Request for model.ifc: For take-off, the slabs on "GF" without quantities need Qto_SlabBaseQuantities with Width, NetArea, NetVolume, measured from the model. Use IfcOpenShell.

First a look at what the model holds.

```python
import ifcopenshell
import ifcopenshell.util.element
import ifcopenshell.util.unit

model = ifcopenshell.open("model.ifc")
print(model.schema)
for unit_type in ("LENGTHUNIT", "AREAUNIT", "VOLUMEUNIT"):
    print(unit_type, ifcopenshell.util.unit.calculate_unit_scale(model, unit_type))
storey = next(s for s in model.by_type("IfcBuildingStorey") if s.Name == "GF")
slabs = [e for e in ifcopenshell.util.element.get_decomposition(storey) if e.is_a("IfcSlab")]
for e in sorted(slabs, key=lambda e: e.id()):
    print(e.id(), e.is_a(), e.Name, list(ifcopenshell.util.element.get_psets(e, qtos_only=True)), sep=" | ")
```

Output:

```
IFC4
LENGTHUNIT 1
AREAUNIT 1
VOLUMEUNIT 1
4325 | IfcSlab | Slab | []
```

```python
import ifcopenshell
import ifcopenshell.api.pset
import ifcopenshell.geom
import ifcopenshell.util.element
import ifcopenshell.util.shape
import ifcopenshell.util.unit

model = ifcopenshell.open("model.ifc")
unit_scale = ifcopenshell.util.unit.calculate_unit_scale(model)
area_scale = ifcopenshell.util.unit.calculate_unit_scale(model, "AREAUNIT")
volume_scale = ifcopenshell.util.unit.calculate_unit_scale(model, "VOLUMEUNIT")
settings = ifcopenshell.geom.settings()

storey = next(s for s in model.by_type("IfcBuildingStorey") if s.Name == "GF")
slabs = [e for e in ifcopenshell.util.element.get_decomposition(storey) if e.is_a("IfcSlab")]

for e in sorted(slabs, key=lambda e: e.id()):
    if ifcopenshell.util.element.get_psets(e, qtos_only=True, should_inherit=False):
        continue
    # Geometry comes back in metres, in the element's own axes.
    shape = ifcopenshell.geom.create_shape(settings, e)
    values = {
        "Width": ifcopenshell.util.shape.get_z(shape.geometry) / unit_scale,
        "NetArea": ifcopenshell.util.shape.get_footprint_area(shape.geometry) / area_scale,
        "NetVolume": ifcopenshell.util.shape.get_volume(shape.geometry) / volume_scale,
    }
    qto = ifcopenshell.api.pset.add_qto(model, product=e, name="Qto_SlabBaseQuantities")
    ifcopenshell.api.pset.edit_qto(model, qto=qto, properties=values)
    print(e.id(), {k: round(v, 3) for k, v in values.items()})

model.write("model_updated.ifc")
```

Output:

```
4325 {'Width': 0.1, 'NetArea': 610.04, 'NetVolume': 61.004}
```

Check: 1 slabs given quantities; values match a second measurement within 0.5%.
